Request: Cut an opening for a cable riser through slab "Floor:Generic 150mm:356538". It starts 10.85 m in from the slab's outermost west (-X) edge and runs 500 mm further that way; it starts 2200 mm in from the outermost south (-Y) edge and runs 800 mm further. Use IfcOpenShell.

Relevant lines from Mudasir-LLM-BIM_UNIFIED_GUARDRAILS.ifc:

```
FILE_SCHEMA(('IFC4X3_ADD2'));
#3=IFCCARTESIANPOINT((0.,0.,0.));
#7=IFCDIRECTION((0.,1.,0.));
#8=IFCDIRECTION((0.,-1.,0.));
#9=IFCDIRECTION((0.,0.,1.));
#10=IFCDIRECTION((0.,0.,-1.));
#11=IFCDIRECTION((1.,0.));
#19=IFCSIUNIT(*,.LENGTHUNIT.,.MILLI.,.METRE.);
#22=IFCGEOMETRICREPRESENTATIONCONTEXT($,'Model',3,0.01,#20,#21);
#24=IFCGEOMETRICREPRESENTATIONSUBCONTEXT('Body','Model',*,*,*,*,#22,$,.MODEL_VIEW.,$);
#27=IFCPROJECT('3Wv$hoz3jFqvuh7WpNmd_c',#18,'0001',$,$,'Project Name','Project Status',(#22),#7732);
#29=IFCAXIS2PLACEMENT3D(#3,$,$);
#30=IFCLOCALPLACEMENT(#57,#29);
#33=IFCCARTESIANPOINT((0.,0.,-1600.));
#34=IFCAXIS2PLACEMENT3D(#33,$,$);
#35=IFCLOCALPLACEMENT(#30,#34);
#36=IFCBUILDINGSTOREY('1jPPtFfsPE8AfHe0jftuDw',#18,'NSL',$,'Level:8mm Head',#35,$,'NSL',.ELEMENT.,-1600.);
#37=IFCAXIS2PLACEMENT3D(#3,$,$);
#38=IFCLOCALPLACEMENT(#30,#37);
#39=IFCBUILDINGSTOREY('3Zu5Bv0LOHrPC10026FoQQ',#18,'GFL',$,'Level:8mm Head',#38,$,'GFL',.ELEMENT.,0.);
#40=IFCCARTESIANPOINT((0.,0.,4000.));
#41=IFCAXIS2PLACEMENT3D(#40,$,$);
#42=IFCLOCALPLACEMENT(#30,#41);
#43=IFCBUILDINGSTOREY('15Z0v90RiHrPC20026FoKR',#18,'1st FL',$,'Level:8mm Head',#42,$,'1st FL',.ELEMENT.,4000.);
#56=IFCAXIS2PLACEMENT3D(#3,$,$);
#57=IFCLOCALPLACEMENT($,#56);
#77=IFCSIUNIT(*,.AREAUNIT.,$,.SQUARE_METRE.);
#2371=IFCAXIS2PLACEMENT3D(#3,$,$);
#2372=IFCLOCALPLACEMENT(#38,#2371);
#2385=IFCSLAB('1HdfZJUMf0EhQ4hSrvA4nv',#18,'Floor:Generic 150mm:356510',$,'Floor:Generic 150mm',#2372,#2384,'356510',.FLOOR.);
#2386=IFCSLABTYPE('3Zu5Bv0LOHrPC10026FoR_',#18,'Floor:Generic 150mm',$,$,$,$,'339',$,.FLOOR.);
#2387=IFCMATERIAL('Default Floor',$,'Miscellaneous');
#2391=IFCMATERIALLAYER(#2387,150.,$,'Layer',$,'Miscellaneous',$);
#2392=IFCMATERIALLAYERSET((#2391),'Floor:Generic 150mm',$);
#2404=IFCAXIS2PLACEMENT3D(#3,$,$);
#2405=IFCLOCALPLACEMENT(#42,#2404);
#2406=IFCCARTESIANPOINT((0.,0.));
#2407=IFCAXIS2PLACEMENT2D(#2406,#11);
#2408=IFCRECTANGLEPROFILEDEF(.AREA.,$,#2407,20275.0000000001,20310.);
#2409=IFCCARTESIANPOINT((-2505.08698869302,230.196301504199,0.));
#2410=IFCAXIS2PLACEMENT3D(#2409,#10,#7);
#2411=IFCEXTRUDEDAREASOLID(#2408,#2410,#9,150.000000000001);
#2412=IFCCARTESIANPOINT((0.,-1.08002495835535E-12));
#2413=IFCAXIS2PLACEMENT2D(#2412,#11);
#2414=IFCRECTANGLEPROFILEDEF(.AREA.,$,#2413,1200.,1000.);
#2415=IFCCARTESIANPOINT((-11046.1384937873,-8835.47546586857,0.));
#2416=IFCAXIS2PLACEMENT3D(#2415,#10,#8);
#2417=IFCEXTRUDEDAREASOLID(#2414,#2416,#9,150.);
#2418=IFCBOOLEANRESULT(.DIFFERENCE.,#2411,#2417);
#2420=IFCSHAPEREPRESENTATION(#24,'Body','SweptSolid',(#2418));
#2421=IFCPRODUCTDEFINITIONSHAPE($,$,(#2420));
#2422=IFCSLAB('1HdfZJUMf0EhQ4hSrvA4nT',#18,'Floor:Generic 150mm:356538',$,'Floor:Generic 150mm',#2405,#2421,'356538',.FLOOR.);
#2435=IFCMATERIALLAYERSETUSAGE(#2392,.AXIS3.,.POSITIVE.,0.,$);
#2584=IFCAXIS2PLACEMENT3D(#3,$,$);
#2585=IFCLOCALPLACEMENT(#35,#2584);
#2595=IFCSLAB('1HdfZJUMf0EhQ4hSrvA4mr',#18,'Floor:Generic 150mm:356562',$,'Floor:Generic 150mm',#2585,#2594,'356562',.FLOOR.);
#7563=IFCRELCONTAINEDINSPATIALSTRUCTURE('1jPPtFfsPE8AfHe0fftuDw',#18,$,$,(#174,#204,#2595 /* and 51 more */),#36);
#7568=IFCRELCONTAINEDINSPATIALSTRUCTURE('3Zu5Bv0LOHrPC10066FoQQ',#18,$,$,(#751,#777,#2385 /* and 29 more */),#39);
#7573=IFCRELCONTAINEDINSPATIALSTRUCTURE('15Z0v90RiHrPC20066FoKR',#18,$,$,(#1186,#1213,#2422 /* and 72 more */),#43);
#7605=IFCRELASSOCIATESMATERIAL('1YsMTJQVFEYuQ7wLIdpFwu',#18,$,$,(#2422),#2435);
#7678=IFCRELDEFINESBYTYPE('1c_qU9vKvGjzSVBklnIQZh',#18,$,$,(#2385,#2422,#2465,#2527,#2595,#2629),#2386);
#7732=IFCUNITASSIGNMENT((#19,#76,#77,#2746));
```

```python
import numpy as np
import ifcopenshell
import ifcopenshell.api.feature
import ifcopenshell.api.geometry
import ifcopenshell.api.root
import ifcopenshell.geom
import ifcopenshell.util.placement
import ifcopenshell.util.representation
import ifcopenshell.util.shape
import ifcopenshell.util.unit

model = ifcopenshell.open("Mudasir-LLM-BIM_UNIFIED_GUARDRAILS.ifc")
unit_scale = ifcopenshell.util.unit.calculate_unit_scale(model)
settings = ifcopenshell.geom.settings()


def volume(element):
    """Net volume in cubic metres, openings subtracted."""
    shape = ifcopenshell.geom.create_shape(settings, element)
    return ifcopenshell.util.shape.get_volume(shape.geometry)


slab = model.by_guid("1HdfZJUMf0EhQ4hSrvA4nT")
before = volume(slab)

# Extent in the slab's own axes, in metres. The edges named are its -X and -Y sides.
slab_shape = ifcopenshell.geom.create_shape(settings, slab)
vertices = ifcopenshell.util.shape.get_vertices(slab_shape.geometry)
x_min, y_min, bottom = vertices.min(axis=0)
top = vertices[:, 2].max()

opening = ifcopenshell.api.root.create_entity(model, ifc_class="IfcOpeningElement", name="Cable riser opening", predefined_type="OPENING")
context = ifcopenshell.util.representation.get_context(model, "Model", "Body", "MODEL_VIEW")
width, depth = 0.5, 0.8
outline = [(0.0, 0.0), (width, 0.0), (width, depth), (0.0, depth), (0.0, 0.0)]
# Overshoot both faces by 50 mm so the cut is clean.
shape = ifcopenshell.api.geometry.add_slab_representation(
    model, context=context, depth=top - bottom + 0.1, polyline=outline
)
ifcopenshell.api.geometry.assign_representation(model, product=opening, representation=shape)

matrix = ifcopenshell.util.placement.get_local_placement(slab.ObjectPlacement)
matrix[:, 3] = matrix @ np.append(np.array([x_min + 10.85, y_min + 2.2, bottom - 0.05]) / unit_scale, 1.0)
ifcopenshell.api.geometry.edit_object_placement(model, product=opening, matrix=matrix, is_si=False)
ifcopenshell.api.feature.add_feature(model, feature=opening, element=slab)

after = volume(slab)

print(f"slab volume {before:.3f} -> {after:.3f} m3")

model.write("Mudasir-LLM-BIM_UNIFIED_GUARDRAILS_rev.ifc")
```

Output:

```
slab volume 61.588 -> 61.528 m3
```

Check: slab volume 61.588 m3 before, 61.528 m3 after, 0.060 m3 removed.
